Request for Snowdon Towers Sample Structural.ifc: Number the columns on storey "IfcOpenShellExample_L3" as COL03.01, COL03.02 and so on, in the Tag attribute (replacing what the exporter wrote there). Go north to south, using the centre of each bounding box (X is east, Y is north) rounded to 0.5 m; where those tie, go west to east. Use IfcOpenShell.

First a look at what the model holds.

```python
import ifcopenshell
import ifcopenshell.util.element
import ifcopenshell.util.placement

model = ifcopenshell.open("Snowdon Towers Sample Structural.ifc")
print(model.schema)
storey = next(s for s in model.by_type("IfcBuildingStorey") if s.Name == "IfcOpenShellExample_L3")
columns = [e for e in ifcopenshell.util.element.get_decomposition(storey) if e.is_a("IfcColumn")]
for e in sorted(columns, key=lambda e: e.id()):
    origin = ifcopenshell.util.placement.get_local_placement(e.ObjectPlacement)[:3, 3]
    print(e.id(), e.Tag, e.Name, origin.round(2) + 0.0, sep=" | ")
```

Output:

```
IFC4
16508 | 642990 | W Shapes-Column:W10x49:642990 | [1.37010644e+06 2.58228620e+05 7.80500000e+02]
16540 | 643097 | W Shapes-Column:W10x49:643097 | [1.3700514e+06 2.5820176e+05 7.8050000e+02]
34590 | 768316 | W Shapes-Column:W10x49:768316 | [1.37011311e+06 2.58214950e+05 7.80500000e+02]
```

```python
import ifcopenshell
import ifcopenshell.geom
import ifcopenshell.util.element
import ifcopenshell.util.shape

model = ifcopenshell.open("Snowdon Towers Sample Structural.ifc")
settings = ifcopenshell.geom.settings()
settings.set("use-world-coords", True)


def centre(element):
    shape = ifcopenshell.geom.create_shape(settings, element)
    return ifcopenshell.util.shape.get_bbox_centroid(shape.geometry)


storey = next(s for s in model.by_type("IfcBuildingStorey") if s.Name == "IfcOpenShellExample_L3")
columns = [e for e in ifcopenshell.util.element.get_decomposition(storey) if e.is_a("IfcColumn")]

# Insertion points can sit at a corner or the storey origin, so sort by the geometry (in metres).
centres = {e: centre(e) for e in columns}
columns.sort(key=lambda e: (-round(centres[e][1] / 0.5), centres[e][0]))

for i, e in enumerate(columns, start=1):
    number = f"COL03.{i:02d}"
    e.Tag = number
    print(e.id(), number)

model.write("Snowdon Towers Sample Structural-out.ifc")
```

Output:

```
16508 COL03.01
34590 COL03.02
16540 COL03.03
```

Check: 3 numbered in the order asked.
